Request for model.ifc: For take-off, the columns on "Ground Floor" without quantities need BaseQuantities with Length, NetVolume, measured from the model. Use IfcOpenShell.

First a look at what the model holds.

```python
import ifcopenshell
import ifcopenshell.util.element
import ifcopenshell.util.unit

model = ifcopenshell.open("model.ifc")
print(model.schema)
for unit_type in ("LENGTHUNIT", "AREAUNIT", "VOLUMEUNIT"):
    print(unit_type, ifcopenshell.util.unit.calculate_unit_scale(model, unit_type))
storey = next(s for s in model.by_type("IfcBuildingStorey") if s.Name == "Ground Floor")
columns = [e for e in ifcopenshell.util.element.get_decomposition(storey) if e.is_a("IfcColumn")]
for e in sorted(columns, key=lambda e: e.id()):
    print(e.id(), e.is_a(), e.Name, list(ifcopenshell.util.element.get_psets(e, qtos_only=True)), sep=" | ")
```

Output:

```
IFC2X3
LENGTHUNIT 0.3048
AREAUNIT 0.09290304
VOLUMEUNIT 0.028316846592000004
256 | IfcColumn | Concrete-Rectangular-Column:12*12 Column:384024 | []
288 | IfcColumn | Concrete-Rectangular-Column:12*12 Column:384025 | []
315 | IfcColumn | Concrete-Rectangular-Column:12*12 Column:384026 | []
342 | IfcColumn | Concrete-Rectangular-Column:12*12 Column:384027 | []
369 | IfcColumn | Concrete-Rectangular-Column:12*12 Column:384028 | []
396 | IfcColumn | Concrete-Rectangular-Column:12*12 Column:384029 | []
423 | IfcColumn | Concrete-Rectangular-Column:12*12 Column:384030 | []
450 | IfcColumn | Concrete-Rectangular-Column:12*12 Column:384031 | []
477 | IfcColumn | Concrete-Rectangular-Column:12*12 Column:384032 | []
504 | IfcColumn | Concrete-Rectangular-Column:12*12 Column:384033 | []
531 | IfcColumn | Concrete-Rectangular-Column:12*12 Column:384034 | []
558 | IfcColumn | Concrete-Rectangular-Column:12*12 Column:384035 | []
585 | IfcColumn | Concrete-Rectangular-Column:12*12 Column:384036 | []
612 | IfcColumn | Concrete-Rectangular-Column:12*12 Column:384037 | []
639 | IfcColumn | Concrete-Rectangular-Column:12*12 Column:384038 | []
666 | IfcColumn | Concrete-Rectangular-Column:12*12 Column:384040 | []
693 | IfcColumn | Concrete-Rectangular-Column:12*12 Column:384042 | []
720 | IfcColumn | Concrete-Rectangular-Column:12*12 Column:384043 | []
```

```python
import ifcopenshell
import ifcopenshell.api.pset
import ifcopenshell.geom
import ifcopenshell.util.element
import ifcopenshell.util.shape
import ifcopenshell.util.unit

model = ifcopenshell.open("model.ifc")
unit_scale = ifcopenshell.util.unit.calculate_unit_scale(model)
volume_scale = ifcopenshell.util.unit.calculate_unit_scale(model, "VOLUMEUNIT")
settings = ifcopenshell.geom.settings()

storey = next(s for s in model.by_type("IfcBuildingStorey") if s.Name == "Ground Floor")
columns = [e for e in ifcopenshell.util.element.get_decomposition(storey) if e.is_a("IfcColumn")]

for e in sorted(columns, key=lambda e: e.id()):
    if ifcopenshell.util.element.get_psets(e, qtos_only=True, should_inherit=False):
        continue
    # Geometry comes back in metres, in the element's own axes.
    shape = ifcopenshell.geom.create_shape(settings, e)
    values = {
        "Length": ifcopenshell.util.shape.get_z(shape.geometry) / unit_scale,
        "NetVolume": ifcopenshell.util.shape.get_volume(shape.geometry) / volume_scale,
    }
    qto = ifcopenshell.api.pset.add_qto(model, product=e, name="BaseQuantities")
    ifcopenshell.api.pset.edit_qto(model, qto=qto, properties=values)
    print(e.id(), {k: round(v, 3) for k, v in values.items()})

model.write("model-out.ifc")
```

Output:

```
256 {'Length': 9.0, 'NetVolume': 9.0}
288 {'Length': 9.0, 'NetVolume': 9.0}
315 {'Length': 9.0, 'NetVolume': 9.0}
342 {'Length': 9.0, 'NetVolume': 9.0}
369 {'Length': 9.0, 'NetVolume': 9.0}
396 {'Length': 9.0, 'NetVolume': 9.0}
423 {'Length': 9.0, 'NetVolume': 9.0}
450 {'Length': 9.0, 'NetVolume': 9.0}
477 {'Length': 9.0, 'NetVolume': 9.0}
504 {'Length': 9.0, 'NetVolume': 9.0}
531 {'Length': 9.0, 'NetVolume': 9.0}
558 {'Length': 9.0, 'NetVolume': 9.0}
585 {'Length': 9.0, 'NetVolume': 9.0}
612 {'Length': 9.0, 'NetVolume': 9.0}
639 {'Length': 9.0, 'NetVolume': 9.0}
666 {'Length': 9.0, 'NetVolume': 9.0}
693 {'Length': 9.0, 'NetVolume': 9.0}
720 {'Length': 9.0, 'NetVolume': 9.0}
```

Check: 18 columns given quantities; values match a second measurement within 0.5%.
